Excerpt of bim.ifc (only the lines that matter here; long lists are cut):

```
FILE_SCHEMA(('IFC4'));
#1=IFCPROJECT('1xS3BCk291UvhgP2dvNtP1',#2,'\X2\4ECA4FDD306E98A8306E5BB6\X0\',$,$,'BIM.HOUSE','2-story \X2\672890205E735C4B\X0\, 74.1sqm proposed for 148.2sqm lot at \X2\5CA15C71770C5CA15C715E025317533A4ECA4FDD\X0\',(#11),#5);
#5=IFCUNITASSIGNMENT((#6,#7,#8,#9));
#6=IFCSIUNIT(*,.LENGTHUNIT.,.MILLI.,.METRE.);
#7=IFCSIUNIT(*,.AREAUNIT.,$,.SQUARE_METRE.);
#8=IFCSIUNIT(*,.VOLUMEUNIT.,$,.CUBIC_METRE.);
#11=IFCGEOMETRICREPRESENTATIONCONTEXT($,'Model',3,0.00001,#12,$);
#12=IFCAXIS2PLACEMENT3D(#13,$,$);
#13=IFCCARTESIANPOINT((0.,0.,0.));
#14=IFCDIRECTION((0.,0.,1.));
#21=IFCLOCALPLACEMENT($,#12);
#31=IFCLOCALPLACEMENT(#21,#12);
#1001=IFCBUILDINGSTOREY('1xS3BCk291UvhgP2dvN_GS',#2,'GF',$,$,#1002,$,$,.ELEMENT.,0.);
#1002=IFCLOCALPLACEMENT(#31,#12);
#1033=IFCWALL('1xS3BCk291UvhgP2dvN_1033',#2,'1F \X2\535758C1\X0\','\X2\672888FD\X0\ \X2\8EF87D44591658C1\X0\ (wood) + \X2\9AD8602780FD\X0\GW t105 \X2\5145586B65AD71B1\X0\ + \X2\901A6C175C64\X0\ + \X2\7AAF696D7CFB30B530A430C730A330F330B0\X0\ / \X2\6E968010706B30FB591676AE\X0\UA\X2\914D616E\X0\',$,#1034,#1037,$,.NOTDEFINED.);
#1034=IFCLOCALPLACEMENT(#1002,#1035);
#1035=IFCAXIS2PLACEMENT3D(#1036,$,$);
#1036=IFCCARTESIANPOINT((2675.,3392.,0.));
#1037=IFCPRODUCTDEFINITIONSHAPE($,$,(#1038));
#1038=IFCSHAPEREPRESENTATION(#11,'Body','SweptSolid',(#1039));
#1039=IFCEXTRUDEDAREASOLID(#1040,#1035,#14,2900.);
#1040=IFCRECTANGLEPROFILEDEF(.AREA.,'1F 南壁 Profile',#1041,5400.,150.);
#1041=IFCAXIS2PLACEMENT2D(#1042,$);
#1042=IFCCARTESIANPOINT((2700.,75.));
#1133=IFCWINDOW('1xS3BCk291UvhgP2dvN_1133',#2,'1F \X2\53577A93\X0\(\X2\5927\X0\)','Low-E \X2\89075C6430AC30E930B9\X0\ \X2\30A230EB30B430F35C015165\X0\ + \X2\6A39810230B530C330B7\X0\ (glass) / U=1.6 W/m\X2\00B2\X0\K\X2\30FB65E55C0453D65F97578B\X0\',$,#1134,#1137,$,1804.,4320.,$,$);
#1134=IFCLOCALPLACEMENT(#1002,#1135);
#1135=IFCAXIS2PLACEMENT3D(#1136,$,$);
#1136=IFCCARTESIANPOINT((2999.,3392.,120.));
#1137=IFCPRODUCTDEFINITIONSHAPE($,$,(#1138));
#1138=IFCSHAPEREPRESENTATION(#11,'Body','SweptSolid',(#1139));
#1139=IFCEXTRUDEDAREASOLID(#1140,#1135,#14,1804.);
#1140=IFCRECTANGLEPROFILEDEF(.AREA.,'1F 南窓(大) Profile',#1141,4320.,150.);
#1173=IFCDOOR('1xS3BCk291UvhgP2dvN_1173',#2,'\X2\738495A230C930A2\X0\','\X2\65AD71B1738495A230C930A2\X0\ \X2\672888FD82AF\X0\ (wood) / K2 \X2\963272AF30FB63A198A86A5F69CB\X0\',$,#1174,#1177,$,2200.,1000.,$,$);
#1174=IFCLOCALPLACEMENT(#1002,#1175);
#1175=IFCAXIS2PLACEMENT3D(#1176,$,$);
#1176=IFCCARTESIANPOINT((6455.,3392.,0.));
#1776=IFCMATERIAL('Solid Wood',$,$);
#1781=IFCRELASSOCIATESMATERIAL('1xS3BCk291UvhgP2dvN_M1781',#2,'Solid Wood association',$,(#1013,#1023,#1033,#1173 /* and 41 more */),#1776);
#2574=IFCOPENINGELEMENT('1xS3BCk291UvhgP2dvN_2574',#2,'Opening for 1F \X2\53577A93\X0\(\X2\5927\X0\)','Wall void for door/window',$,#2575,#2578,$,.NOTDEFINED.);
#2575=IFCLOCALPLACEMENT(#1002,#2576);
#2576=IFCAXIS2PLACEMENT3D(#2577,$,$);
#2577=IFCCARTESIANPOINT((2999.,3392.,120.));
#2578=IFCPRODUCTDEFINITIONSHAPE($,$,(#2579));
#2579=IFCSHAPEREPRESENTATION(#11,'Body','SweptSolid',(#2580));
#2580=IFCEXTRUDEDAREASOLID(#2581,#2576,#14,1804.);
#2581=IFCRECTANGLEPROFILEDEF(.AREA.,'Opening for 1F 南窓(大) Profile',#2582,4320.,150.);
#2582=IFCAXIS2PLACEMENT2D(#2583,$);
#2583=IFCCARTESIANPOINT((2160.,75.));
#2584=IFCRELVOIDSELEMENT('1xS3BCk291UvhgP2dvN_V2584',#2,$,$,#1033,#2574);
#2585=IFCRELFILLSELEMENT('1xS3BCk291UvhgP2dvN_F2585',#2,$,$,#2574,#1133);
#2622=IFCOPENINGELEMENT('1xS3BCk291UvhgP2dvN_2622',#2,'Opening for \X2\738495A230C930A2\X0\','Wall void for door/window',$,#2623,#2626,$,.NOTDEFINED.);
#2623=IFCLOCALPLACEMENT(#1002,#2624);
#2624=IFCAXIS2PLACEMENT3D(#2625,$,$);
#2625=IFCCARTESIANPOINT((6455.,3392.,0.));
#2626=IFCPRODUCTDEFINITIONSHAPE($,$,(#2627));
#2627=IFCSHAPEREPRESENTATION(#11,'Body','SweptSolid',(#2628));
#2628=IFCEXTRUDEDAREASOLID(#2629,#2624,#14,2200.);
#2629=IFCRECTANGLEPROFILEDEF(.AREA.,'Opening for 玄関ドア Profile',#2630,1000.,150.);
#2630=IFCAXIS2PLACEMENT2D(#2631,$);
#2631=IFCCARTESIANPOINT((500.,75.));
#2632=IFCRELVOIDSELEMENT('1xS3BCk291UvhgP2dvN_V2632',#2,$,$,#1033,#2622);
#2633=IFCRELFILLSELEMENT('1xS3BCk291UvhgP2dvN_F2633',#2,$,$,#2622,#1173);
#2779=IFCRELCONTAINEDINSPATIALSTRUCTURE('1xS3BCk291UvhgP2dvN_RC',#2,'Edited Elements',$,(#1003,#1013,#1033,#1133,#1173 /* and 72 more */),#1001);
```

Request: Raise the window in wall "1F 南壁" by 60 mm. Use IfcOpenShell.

```python
import numpy as np
import ifcopenshell
import ifcopenshell.api.geometry
import ifcopenshell.util.placement
import ifcopenshell.util.unit

model = ifcopenshell.open("bim.ifc")
unit_scale = ifcopenshell.util.unit.calculate_unit_scale(model)

window = model.by_guid("1xS3BCk291UvhgP2dvN_1133")
opening = window.FillsVoids[0].RelatingOpeningElement
dz = 0.06 / unit_scale

shift = np.array([0.0, 0.0, dz])
# The window is not placed relative to its opening, so move both.
for product in (opening, window):
    matrix = ifcopenshell.util.placement.get_local_placement(product.ObjectPlacement)
    matrix[:3, 3] += shift
    ifcopenshell.api.geometry.edit_object_placement(model, product=product, matrix=matrix, is_si=False)

print(f"moved by {dz * unit_scale:+.3f} m")

model.write("bim_rev.ifc")
```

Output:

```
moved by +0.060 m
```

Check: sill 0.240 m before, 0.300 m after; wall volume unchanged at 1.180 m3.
